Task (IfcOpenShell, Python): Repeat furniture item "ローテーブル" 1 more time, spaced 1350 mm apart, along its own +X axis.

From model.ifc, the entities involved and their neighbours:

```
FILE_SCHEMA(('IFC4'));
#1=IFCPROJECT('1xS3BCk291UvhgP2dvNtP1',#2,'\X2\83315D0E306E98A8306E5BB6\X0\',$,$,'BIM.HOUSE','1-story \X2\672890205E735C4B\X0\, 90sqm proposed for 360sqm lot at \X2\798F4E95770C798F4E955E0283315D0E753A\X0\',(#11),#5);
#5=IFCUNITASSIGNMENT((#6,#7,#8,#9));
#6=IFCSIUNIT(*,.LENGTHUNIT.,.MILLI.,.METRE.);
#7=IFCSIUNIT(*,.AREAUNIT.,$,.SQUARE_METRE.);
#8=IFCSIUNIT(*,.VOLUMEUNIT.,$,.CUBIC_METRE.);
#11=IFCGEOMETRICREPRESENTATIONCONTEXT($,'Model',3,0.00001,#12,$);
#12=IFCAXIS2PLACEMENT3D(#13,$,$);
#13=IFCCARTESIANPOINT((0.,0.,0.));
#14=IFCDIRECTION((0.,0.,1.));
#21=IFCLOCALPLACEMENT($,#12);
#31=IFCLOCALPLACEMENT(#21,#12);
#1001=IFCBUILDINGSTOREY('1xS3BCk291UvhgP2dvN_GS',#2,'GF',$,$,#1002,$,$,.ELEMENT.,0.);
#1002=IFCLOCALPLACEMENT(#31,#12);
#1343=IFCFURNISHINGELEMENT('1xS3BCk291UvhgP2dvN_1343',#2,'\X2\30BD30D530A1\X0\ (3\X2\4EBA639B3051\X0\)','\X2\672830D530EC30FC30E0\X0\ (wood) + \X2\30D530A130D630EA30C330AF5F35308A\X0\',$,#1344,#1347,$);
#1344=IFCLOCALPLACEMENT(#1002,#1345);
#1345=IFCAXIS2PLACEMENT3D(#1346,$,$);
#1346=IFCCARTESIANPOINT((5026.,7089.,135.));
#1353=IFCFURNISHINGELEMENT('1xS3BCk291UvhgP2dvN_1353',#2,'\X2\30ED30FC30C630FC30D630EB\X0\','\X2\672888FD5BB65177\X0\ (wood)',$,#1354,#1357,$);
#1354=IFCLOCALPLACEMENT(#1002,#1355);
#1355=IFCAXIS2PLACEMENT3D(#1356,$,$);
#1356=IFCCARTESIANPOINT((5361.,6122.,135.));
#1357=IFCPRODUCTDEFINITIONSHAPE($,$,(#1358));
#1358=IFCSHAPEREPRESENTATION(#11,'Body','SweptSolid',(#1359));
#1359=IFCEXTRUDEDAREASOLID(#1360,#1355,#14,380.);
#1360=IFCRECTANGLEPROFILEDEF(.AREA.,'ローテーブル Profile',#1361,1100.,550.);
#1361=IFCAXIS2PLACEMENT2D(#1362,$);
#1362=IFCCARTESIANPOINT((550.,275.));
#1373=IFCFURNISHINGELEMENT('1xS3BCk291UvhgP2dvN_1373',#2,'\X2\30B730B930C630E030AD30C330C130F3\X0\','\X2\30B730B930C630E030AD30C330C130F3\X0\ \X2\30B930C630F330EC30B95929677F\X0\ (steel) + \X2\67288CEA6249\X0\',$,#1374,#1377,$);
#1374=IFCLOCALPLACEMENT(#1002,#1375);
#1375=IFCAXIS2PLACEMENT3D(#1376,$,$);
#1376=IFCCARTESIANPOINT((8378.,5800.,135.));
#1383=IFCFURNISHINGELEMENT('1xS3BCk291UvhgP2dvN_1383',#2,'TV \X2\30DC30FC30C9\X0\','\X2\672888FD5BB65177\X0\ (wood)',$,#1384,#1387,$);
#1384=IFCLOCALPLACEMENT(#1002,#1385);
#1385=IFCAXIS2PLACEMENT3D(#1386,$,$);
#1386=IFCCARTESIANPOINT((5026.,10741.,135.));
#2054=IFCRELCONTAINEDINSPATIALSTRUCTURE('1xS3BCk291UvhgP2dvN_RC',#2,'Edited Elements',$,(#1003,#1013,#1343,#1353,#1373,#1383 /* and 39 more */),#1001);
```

```python
import ifcopenshell
import ifcopenshell.api.geometry
import ifcopenshell.api.root
import ifcopenshell.util.element
import ifcopenshell.util.placement
import ifcopenshell.util.unit

model = ifcopenshell.open("model.ifc")
unit_scale = ifcopenshell.util.unit.calculate_unit_scale(model)


def reuse_history(source, copy):
    """copy_class also copies each property set's owner history, people and application; keep the originals."""
    for rel in copy.IsDefinedBy:
        if rel.is_a("IfcRelDefinesByProperties") and (history := rel.RelatingPropertyDefinition.OwnerHistory):
            rel.RelatingPropertyDefinition.OwnerHistory = source.OwnerHistory
            ifcopenshell.util.element.remove_deep2(model, history)


source = model.by_guid("1xS3BCk291UvhgP2dvN_1353")
base = ifcopenshell.util.placement.get_local_placement(source.ObjectPlacement)
step = base[:3, 0] * 1.35 / unit_scale

for i in range(1, 2):
    copy = ifcopenshell.api.root.copy_class(model, product=source)
    copy.Representation = ifcopenshell.util.element.copy_deep(
        model, source.Representation, exclude=["IfcGeometricRepresentationContext", "IfcRepresentationMap"]
    )
    reuse_history(source, copy)
    matrix = base.copy()
    matrix[:3, 3] += i * step
    print("added at", matrix[:3, 3].round(3) + 0.0)
    ifcopenshell.api.geometry.edit_object_placement(model, product=copy, matrix=matrix, is_si=False)

model.write("model_edited.ifc")
```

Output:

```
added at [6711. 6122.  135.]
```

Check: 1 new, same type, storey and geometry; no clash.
